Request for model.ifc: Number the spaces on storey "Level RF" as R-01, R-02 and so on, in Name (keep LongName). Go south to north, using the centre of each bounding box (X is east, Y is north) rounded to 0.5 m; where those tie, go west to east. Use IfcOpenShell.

First a look at what the model holds.

```python
import ifcopenshell
import ifcopenshell.util.element
import ifcopenshell.util.placement

model = ifcopenshell.open("model.ifc")
print(model.schema)
storey = next(s for s in model.by_type("IfcBuildingStorey") if s.Name == "Level RF")
spaces = [e for e in ifcopenshell.util.element.get_decomposition(storey) if e.is_a("IfcSpace")]
for e in sorted(spaces, key=lambda e: e.id()):
    origin = ifcopenshell.util.placement.get_local_placement(e.ObjectPlacement)[:3, 3]
    print(e.id(), e.Name, e.LongName, origin.round(2) + 0.0, sep=" | ")
```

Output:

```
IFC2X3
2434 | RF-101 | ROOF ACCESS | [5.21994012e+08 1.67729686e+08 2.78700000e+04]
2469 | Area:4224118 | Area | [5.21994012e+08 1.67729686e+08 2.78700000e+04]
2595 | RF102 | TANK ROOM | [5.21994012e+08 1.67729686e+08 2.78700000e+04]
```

```python
import ifcopenshell
import ifcopenshell.geom
import ifcopenshell.util.element
import ifcopenshell.util.shape

model = ifcopenshell.open("model.ifc")
settings = ifcopenshell.geom.settings()
settings.set("use-world-coords", True)


def centre(element):
    shape = ifcopenshell.geom.create_shape(settings, element)
    return ifcopenshell.util.shape.get_bbox_centroid(shape.geometry)


storey = next(s for s in model.by_type("IfcBuildingStorey") if s.Name == "Level RF")
spaces = [e for e in ifcopenshell.util.element.get_decomposition(storey) if e.is_a("IfcSpace")]

# Insertion points can sit at a corner or the storey origin, so sort by the geometry (in metres).
centres = {e: centre(e) for e in spaces}
spaces.sort(key=lambda e: (round(centres[e][1] / 0.5), centres[e][0]))

for i, e in enumerate(spaces, start=1):
    number = f"R-{i:02d}"
    e.Name = number
    print(e.id(), number)

model.write("model_updated.ifc")
```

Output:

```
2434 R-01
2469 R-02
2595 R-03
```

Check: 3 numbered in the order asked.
